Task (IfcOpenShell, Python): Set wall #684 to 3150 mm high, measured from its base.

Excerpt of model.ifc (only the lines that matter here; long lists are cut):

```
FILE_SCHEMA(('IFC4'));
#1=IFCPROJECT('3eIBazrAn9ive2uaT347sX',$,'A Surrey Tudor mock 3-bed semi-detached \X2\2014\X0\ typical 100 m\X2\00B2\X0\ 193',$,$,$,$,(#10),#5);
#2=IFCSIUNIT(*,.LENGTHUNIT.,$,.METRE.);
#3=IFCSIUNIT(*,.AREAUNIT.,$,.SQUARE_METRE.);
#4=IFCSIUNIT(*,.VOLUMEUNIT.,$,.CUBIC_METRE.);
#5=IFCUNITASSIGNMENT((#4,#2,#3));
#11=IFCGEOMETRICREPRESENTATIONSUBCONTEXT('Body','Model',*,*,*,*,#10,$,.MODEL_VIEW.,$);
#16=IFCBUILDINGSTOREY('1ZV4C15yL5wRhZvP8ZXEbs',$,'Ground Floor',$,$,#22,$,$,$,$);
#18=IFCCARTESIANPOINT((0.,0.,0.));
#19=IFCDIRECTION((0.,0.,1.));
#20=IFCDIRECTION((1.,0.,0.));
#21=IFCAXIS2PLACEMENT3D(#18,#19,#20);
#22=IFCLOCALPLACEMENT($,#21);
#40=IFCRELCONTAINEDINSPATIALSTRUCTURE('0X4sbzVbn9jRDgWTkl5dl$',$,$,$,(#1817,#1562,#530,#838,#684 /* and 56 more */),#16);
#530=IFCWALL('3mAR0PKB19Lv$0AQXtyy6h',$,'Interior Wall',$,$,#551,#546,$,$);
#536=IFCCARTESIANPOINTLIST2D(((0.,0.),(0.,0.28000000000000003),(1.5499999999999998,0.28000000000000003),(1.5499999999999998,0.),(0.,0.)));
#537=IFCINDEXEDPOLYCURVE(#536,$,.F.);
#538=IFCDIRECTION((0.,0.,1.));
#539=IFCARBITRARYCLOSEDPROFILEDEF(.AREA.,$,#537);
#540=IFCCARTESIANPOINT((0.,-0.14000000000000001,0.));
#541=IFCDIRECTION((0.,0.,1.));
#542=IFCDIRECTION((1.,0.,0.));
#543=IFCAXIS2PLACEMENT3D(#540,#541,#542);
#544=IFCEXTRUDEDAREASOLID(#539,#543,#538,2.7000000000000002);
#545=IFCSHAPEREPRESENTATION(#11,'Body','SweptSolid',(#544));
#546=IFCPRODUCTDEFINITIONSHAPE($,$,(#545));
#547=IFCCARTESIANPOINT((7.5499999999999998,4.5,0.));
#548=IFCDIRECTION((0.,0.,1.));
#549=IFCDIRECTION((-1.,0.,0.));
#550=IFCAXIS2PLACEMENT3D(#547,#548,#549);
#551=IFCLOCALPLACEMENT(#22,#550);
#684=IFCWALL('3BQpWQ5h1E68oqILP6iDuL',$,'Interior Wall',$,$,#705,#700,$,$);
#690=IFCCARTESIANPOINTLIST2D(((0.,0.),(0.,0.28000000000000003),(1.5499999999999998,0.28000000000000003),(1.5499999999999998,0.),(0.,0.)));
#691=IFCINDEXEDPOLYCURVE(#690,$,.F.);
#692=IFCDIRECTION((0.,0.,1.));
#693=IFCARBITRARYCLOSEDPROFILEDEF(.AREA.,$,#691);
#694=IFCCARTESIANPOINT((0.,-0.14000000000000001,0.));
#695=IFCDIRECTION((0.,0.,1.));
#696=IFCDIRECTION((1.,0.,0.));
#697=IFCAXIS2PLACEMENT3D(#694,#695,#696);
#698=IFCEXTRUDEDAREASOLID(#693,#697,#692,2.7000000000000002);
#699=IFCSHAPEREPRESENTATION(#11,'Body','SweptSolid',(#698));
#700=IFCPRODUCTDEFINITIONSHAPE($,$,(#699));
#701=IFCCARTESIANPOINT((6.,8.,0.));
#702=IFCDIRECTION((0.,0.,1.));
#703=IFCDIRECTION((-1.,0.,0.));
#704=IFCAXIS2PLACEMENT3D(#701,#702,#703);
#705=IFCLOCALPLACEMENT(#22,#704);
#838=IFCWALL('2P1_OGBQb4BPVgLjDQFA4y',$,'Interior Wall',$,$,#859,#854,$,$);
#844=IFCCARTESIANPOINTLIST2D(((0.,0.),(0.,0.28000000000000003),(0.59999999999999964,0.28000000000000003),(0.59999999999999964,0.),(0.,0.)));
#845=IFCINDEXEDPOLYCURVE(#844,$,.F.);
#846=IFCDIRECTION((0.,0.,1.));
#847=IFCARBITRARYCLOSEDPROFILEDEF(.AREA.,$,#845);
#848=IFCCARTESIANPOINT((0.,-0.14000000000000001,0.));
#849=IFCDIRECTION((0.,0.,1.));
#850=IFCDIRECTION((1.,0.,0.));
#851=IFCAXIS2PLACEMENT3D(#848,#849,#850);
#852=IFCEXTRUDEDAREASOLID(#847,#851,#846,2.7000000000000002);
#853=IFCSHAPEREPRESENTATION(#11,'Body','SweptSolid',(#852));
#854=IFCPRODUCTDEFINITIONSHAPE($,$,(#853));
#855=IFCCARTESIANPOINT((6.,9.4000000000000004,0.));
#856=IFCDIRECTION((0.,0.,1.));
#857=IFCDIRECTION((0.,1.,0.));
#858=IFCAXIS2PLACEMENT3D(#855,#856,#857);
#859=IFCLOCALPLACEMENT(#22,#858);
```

```python
import ifcopenshell
import ifcopenshell.geom
import ifcopenshell.util.representation
import ifcopenshell.util.shape
import ifcopenshell.util.unit

model = ifcopenshell.open("model.ifc")
unit_scale = ifcopenshell.util.unit.calculate_unit_scale(model)
settings = ifcopenshell.geom.settings()


def volume(element):
    """Net volume in cubic metres, openings subtracted."""
    shape = ifcopenshell.geom.create_shape(settings, element)
    return ifcopenshell.util.shape.get_volume(shape.geometry)


wall = model.by_guid("3BQpWQ5h1E68oqILP6iDuL")
before = volume(wall)

body = ifcopenshell.util.representation.get_representation(wall, "Model", "Body")
solid = body.Items[0]
old_height = solid.Depth
solid.Depth = 3.15 / unit_scale
after = volume(wall)

print(f"height {old_height:g} -> {solid.Depth:g}, volume {before:.3f} -> {after:.3f} m3")

model.write("model_edited.ifc")
```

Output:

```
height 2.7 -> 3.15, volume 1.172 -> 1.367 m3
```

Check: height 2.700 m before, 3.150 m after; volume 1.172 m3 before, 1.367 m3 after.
